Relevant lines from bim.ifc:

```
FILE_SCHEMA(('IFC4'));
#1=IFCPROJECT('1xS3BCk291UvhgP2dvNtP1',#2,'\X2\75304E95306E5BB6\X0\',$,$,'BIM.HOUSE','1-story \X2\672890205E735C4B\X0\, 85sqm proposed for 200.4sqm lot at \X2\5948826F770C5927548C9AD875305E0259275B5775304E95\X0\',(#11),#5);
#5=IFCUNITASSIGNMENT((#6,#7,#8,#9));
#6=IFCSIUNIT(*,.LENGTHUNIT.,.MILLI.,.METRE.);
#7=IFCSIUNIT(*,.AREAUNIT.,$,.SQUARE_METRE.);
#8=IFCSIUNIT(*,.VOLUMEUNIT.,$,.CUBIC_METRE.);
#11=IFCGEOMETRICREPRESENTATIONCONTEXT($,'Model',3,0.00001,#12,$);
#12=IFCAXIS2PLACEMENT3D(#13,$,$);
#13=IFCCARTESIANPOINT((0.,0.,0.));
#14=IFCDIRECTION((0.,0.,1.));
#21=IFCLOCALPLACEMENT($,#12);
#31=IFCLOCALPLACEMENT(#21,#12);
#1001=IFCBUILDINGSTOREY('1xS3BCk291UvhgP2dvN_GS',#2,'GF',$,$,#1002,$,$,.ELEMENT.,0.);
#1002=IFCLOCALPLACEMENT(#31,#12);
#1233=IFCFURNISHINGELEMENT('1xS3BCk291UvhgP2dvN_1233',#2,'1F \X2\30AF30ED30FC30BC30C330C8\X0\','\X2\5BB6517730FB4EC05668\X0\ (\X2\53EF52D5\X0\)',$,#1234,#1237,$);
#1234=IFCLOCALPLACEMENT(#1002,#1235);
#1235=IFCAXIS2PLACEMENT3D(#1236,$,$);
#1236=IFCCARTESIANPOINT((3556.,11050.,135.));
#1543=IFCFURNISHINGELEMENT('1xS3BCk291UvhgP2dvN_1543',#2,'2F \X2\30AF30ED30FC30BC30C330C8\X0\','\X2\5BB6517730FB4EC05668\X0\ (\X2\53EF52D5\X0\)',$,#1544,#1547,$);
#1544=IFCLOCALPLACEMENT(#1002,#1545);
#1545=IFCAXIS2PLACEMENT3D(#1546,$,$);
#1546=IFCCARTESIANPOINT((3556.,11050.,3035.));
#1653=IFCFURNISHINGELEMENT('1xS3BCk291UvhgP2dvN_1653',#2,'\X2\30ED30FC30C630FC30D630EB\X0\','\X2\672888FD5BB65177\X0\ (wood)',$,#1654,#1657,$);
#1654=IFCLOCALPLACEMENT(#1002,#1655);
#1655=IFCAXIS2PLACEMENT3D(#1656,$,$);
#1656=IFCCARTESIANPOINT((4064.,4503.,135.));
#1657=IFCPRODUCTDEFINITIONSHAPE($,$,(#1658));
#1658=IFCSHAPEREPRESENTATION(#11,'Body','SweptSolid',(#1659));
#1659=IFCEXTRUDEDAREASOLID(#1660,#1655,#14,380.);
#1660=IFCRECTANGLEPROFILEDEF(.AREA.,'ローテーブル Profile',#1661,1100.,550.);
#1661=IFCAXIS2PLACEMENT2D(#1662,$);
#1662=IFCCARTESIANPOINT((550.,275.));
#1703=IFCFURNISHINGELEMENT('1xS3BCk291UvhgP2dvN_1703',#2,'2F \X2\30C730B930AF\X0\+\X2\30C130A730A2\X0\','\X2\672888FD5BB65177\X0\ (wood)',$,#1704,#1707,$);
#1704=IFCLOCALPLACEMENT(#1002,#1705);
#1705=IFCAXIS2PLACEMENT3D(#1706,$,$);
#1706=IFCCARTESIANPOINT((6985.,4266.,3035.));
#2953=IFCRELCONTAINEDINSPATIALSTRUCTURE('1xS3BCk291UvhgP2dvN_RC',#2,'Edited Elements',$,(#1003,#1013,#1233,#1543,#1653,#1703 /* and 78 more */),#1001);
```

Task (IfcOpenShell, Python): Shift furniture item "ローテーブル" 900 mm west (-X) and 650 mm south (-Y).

```python
import ifcopenshell
import ifcopenshell.api.geometry
import ifcopenshell.util.placement

model = ifcopenshell.open("bim.ifc")

item = model.by_guid("1xS3BCk291UvhgP2dvN_1653")
matrix = ifcopenshell.util.placement.get_local_placement(item.ObjectPlacement)
matrix[0, 3] -= 900.0
matrix[1, 3] -= 650.0
ifcopenshell.api.geometry.edit_object_placement(model, product=item, matrix=matrix, is_si=False)

print(ifcopenshell.util.placement.get_local_placement(item.ObjectPlacement).round(3) + 0.0)

model.write("bim_rev.ifc")
```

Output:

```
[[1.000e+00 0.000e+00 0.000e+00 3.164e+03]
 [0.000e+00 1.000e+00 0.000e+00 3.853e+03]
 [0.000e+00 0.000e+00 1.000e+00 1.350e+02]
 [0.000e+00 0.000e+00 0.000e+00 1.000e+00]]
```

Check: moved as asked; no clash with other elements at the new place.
